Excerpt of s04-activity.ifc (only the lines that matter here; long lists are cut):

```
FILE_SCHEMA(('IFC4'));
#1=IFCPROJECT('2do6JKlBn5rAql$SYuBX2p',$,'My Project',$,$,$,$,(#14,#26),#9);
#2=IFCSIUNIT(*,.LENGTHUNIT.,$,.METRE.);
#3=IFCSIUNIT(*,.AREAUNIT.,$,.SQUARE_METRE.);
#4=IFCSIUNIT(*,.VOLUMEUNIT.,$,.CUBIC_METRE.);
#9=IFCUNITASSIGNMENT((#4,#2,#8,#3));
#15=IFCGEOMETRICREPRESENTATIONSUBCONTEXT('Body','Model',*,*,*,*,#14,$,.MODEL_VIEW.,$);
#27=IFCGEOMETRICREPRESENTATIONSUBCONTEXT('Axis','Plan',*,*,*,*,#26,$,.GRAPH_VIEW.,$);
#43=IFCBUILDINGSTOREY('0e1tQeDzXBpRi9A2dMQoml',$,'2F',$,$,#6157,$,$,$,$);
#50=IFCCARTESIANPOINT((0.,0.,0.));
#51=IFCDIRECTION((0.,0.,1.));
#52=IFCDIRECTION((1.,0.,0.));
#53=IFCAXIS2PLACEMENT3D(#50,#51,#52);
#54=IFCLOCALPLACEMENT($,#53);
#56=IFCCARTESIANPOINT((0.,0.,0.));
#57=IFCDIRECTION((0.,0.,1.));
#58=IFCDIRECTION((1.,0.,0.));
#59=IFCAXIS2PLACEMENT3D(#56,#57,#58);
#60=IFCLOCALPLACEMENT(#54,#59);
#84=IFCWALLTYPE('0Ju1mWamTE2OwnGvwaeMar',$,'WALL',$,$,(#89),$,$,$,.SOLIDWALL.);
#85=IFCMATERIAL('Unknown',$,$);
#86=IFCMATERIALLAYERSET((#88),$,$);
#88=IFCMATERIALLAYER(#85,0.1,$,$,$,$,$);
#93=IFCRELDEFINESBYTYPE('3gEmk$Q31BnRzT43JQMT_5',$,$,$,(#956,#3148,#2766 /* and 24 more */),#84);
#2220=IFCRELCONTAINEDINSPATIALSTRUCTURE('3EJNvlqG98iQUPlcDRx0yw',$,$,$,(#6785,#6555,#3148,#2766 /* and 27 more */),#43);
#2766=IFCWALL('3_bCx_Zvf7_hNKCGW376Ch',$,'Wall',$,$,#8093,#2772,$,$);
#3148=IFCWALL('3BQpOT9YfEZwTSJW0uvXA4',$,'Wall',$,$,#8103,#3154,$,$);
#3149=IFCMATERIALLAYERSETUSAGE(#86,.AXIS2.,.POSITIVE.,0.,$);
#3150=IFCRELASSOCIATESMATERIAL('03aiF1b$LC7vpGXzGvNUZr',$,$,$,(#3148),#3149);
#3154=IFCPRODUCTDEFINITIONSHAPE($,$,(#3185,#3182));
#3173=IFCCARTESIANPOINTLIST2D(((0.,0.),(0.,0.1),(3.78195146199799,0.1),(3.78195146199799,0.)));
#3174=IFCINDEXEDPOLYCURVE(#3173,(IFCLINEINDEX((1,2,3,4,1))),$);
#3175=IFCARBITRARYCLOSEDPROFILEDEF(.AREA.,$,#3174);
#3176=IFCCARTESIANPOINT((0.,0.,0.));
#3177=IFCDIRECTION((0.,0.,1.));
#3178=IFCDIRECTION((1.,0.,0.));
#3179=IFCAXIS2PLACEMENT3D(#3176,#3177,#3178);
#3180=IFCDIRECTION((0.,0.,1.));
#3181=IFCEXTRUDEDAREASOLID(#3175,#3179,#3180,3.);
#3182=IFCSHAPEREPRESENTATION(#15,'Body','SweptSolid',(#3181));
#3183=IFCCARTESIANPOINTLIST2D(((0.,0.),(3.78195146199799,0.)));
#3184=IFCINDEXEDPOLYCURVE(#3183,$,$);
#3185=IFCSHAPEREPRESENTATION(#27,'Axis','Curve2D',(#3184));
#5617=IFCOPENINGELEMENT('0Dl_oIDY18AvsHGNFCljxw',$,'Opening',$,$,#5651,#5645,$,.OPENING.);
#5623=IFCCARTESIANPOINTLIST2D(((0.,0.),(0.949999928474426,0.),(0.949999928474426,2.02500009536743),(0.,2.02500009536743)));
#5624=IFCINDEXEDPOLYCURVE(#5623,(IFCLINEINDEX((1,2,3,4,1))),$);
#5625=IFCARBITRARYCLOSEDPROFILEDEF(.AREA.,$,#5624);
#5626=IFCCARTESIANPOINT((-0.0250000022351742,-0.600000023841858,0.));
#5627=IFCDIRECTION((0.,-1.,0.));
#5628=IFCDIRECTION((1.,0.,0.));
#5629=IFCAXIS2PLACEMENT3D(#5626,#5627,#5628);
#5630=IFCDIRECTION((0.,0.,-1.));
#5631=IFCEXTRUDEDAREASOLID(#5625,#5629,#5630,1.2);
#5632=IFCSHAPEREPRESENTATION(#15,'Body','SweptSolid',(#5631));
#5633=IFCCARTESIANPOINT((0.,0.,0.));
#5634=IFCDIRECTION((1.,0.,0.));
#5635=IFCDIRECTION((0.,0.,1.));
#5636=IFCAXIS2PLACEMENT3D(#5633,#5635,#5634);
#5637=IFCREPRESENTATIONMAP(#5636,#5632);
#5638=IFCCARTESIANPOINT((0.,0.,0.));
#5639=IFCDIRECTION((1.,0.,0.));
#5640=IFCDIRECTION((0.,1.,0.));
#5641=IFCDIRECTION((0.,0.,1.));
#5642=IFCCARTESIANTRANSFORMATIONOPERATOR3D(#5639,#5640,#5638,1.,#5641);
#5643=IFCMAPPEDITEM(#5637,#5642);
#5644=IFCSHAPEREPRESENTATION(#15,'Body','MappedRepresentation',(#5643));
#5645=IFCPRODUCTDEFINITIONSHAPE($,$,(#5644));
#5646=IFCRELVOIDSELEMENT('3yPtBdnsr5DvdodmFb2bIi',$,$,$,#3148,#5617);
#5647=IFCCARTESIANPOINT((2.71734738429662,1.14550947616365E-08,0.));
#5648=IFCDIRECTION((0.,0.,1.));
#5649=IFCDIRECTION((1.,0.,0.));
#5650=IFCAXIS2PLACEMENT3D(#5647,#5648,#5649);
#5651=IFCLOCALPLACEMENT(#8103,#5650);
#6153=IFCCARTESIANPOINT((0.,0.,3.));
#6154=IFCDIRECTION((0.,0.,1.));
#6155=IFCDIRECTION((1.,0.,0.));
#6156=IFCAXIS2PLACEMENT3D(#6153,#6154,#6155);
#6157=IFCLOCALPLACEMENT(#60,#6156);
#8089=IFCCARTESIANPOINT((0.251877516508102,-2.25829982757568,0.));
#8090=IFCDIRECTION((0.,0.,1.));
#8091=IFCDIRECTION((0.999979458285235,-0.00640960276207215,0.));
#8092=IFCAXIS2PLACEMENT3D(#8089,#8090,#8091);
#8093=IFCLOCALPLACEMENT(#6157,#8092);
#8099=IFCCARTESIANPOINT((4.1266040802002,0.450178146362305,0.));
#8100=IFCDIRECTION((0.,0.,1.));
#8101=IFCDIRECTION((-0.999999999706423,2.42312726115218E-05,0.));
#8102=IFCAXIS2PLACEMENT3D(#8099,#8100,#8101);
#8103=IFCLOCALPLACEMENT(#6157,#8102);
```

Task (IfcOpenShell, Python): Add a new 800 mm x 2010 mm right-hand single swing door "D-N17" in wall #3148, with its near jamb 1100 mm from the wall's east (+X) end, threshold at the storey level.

```python
import numpy as np
import ifcopenshell
import ifcopenshell.api.feature
import ifcopenshell.api.geometry
import ifcopenshell.api.root
import ifcopenshell.api.spatial
import ifcopenshell.geom
import ifcopenshell.util.element
import ifcopenshell.util.placement
import ifcopenshell.util.representation
import ifcopenshell.util.shape
import ifcopenshell.util.unit

model = ifcopenshell.open("s04-activity.ifc")
unit_scale = ifcopenshell.util.unit.calculate_unit_scale(model)
settings = ifcopenshell.geom.settings()


def volume(element):
    """Net volume in cubic metres, openings subtracted."""
    shape = ifcopenshell.geom.create_shape(settings, element)
    return ifcopenshell.util.shape.get_volume(shape.geometry)


wall = model.by_id(3148)
storey = ifcopenshell.util.element.get_container(wall, ifc_class="IfcBuildingStorey")
context = ifcopenshell.util.representation.get_context(model, "Model", "Body", "MODEL_VIEW")
before = volume(wall)

width, height, from_end, sill = 0.8, 2.01, 1.1, 0.0  # metres

# The wall runs along its own X axis, and the end named is its -X end.
wall_shape = ifcopenshell.geom.create_shape(settings, wall)
x, y, z = ifcopenshell.util.shape.get_vertices(wall_shape.geometry).T
start = x.min() + from_end
face, thickness = float(y.min()), float(y.max() - y.min())
wall_matrix = ifcopenshell.util.placement.get_local_placement(wall.ObjectPlacement)
level = ifcopenshell.util.placement.get_local_placement(storey.ObjectPlacement)[2, 3]


def in_wall(x, y):
    """Placement at x, y metres in the wall's axes, at sill height."""
    matrix = wall_matrix.copy()
    matrix[:, 3] = wall_matrix @ np.array([x / unit_scale, y / unit_scale, 0.0, 1.0])
    matrix[2, 3] = level + sill / unit_scale
    return matrix


# Opening: a box that overshoots both wall faces by 50 mm.
opening = ifcopenshell.api.root.create_entity(model, ifc_class="IfcOpeningElement", predefined_type="OPENING")
box = ifcopenshell.api.geometry.add_wall_representation(
    model, context=context, length=width, height=height, thickness=thickness + 0.1
)
ifcopenshell.api.geometry.assign_representation(model, product=opening, representation=box)
ifcopenshell.api.geometry.edit_object_placement(model, product=opening, matrix=in_wall(start, face - 0.05), is_si=False)
ifcopenshell.api.feature.add_feature(model, feature=opening, element=wall)

door = ifcopenshell.api.root.create_entity(model, ifc_class="IfcDoor", name="D-N17", predefined_type="DOOR")
door.OverallWidth, door.OverallHeight = width / unit_scale, height / unit_scale
door.OperationType = "SINGLE_SWING_RIGHT"
body = ifcopenshell.api.geometry.add_door_representation(
    model,
    context=context,
    overall_width=door.OverallWidth,
    overall_height=door.OverallHeight,
    operation_type="SINGLE_SWING_RIGHT",
    lining_properties={"LiningDepth": thickness / unit_scale, "ThresholdDepth": thickness / unit_scale},
)
ifcopenshell.api.geometry.assign_representation(model, product=door, representation=body)
ifcopenshell.api.spatial.assign_container(model, products=[door], relating_structure=storey)
ifcopenshell.api.feature.add_filling(model, opening=opening, element=door)

# The lining spans the wall, so the door starts at the wall face.
ifcopenshell.api.geometry.edit_object_placement(model, product=door, matrix=in_wall(start, face), is_si=False)

after = volume(wall)

print(f"wall volume {before:.3f} -> {after:.3f} m3")

model.write("s04-activity_rev.ifc")
```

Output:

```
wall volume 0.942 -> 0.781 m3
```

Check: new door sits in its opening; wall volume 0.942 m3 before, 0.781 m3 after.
